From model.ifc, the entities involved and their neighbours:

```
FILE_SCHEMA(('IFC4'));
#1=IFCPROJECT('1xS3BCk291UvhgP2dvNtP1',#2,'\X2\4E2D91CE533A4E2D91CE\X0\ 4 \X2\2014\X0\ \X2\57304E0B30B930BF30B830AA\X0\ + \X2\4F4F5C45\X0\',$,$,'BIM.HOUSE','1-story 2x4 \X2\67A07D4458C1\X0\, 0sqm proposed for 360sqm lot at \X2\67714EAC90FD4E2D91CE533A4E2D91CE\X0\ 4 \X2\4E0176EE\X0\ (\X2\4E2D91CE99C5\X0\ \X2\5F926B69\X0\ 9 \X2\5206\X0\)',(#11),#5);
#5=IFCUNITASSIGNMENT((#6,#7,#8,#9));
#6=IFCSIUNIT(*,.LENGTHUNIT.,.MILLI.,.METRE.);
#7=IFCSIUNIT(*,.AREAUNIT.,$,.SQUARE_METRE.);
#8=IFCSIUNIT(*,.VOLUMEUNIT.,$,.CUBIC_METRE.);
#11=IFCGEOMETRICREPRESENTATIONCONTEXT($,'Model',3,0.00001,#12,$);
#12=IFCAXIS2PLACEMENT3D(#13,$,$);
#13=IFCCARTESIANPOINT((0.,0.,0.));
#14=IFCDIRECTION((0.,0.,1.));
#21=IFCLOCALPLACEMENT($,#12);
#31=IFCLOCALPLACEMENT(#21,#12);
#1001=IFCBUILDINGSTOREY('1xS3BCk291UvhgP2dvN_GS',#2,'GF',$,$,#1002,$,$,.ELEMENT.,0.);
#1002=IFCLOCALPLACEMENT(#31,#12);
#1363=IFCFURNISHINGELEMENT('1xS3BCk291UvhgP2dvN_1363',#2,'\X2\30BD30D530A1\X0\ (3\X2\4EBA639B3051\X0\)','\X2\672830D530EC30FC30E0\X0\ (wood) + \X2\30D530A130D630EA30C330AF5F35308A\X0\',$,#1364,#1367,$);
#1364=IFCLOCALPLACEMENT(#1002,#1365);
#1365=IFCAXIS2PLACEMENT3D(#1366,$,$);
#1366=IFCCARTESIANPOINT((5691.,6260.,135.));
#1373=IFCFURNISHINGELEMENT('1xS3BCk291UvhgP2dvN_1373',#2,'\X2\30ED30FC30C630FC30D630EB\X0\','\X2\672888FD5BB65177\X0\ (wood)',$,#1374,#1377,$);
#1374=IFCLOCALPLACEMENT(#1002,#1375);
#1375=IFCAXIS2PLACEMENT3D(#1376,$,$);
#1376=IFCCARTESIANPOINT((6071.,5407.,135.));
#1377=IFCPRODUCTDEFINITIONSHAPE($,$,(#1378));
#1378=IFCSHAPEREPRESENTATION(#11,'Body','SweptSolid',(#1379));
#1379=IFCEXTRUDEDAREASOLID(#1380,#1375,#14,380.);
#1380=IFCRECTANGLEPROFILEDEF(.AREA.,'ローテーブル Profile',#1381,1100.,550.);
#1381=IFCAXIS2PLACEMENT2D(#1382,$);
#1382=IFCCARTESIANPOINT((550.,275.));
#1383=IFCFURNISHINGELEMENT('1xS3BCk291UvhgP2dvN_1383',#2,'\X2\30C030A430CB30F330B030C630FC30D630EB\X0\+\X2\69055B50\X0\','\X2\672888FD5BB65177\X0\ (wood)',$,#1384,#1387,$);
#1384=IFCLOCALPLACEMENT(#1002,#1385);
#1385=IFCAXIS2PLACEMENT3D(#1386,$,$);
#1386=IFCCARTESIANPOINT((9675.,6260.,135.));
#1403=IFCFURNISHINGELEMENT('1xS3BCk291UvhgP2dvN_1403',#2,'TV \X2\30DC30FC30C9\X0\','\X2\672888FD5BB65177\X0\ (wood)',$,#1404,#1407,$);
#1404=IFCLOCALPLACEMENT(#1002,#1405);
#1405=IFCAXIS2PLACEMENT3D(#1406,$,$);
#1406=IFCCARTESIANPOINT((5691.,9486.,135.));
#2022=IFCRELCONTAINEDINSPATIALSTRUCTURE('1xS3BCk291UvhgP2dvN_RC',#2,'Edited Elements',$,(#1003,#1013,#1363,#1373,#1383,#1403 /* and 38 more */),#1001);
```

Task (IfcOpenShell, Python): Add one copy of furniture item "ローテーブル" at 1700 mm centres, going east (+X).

```python
import numpy as np
import ifcopenshell
import ifcopenshell.api.geometry
import ifcopenshell.api.root
import ifcopenshell.util.element
import ifcopenshell.util.placement
import ifcopenshell.util.unit

model = ifcopenshell.open("model.ifc")
unit_scale = ifcopenshell.util.unit.calculate_unit_scale(model)


def reuse_history(source, copy):
    """copy_class also copies each property set's owner history, people and application; keep the originals."""
    for rel in copy.IsDefinedBy:
        if rel.is_a("IfcRelDefinesByProperties") and (history := rel.RelatingPropertyDefinition.OwnerHistory):
            rel.RelatingPropertyDefinition.OwnerHistory = source.OwnerHistory
            ifcopenshell.util.element.remove_deep2(model, history)


source = model.by_guid("1xS3BCk291UvhgP2dvN_1373")
base = ifcopenshell.util.placement.get_local_placement(source.ObjectPlacement)
step = np.array([1.0, 0.0, 0.0]) * 1.7 / unit_scale

for i in range(1, 2):
    copy = ifcopenshell.api.root.copy_class(model, product=source)
    copy.Representation = ifcopenshell.util.element.copy_deep(
        model, source.Representation, exclude=["IfcGeometricRepresentationContext", "IfcRepresentationMap"]
    )
    reuse_history(source, copy)
    matrix = base.copy()
    matrix[:3, 3] += i * step
    print("added at", matrix[:3, 3].round(3) + 0.0)
    ifcopenshell.api.geometry.edit_object_placement(model, product=copy, matrix=matrix, is_si=False)

model.write("model_updated.ifc")
```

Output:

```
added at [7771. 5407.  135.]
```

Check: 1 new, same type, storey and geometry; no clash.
